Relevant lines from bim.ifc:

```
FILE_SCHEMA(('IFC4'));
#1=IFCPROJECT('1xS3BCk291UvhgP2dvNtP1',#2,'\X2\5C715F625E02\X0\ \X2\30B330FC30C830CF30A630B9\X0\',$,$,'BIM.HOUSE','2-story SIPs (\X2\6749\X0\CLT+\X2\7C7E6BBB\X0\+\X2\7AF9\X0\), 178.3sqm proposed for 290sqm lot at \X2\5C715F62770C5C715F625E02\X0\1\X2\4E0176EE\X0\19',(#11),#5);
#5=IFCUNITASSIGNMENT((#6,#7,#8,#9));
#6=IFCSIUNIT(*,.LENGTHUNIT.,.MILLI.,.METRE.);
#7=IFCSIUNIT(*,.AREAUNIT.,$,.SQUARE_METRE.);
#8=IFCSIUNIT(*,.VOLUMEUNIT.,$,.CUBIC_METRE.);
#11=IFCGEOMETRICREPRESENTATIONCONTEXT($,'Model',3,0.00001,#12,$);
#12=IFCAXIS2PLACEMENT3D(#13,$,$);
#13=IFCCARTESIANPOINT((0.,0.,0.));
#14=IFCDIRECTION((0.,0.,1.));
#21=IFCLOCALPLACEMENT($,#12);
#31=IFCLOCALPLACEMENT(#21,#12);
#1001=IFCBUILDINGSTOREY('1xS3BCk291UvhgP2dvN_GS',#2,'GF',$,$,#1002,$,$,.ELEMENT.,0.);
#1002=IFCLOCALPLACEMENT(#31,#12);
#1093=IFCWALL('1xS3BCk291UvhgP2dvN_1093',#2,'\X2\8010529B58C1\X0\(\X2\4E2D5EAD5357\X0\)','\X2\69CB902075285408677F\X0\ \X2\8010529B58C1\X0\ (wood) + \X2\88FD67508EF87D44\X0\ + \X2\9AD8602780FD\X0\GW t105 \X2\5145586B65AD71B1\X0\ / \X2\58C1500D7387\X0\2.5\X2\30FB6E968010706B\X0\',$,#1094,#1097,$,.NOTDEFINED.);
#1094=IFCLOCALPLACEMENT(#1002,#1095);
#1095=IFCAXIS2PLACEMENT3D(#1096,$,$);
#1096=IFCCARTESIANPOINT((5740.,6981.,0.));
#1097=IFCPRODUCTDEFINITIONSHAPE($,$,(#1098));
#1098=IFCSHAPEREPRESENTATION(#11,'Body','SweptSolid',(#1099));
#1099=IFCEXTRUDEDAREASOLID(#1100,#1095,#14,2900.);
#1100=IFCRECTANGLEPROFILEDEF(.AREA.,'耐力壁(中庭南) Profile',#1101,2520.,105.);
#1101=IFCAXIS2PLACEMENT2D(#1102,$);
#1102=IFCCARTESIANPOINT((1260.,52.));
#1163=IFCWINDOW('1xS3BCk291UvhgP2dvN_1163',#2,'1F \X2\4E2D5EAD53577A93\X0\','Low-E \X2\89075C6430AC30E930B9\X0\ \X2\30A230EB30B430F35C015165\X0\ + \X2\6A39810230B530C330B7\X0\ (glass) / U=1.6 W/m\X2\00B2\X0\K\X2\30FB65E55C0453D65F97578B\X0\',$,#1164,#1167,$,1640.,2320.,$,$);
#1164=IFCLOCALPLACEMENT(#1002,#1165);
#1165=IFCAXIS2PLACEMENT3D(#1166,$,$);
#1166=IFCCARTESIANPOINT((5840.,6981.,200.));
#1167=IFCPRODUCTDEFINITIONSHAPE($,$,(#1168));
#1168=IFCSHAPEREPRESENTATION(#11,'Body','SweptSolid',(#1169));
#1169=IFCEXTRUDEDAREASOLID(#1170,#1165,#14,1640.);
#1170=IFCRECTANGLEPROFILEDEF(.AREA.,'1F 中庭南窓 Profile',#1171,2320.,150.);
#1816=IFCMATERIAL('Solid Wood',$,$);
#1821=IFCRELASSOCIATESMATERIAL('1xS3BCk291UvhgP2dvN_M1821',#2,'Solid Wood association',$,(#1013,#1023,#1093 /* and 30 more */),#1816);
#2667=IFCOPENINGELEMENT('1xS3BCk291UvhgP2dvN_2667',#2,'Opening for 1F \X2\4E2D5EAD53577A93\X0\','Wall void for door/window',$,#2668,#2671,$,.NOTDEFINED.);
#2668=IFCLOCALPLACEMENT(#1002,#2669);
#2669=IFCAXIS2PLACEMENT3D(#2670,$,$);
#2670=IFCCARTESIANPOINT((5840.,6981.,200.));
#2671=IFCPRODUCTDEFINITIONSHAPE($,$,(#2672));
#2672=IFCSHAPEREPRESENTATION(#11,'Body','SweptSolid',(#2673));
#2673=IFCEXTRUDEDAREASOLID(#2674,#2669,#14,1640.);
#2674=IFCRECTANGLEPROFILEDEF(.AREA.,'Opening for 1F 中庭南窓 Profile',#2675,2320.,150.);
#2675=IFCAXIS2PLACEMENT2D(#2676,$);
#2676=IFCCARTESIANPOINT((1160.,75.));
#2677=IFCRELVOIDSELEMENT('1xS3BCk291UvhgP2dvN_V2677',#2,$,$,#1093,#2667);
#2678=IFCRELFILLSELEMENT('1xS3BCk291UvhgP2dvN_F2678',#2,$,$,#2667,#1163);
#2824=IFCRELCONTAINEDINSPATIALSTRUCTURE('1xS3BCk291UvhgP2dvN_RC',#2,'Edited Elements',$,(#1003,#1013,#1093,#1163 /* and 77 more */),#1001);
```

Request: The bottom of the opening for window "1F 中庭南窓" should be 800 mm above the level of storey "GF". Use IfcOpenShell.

```python
import numpy as np
import ifcopenshell
import ifcopenshell.api.geometry
import ifcopenshell.geom
import ifcopenshell.util.element
import ifcopenshell.util.placement
import ifcopenshell.util.shape
import ifcopenshell.util.unit

model = ifcopenshell.open("bim.ifc")
unit_scale = ifcopenshell.util.unit.calculate_unit_scale(model)

window = model.by_guid("1xS3BCk291UvhgP2dvN_1163")
opening = window.FillsVoids[0].RelatingOpeningElement
storey = ifcopenshell.util.element.get_container(window, ifc_class="IfcBuildingStorey")
level = ifcopenshell.util.placement.get_local_placement(storey.ObjectPlacement)[2, 3]

# The opening's origin need not be at the sill, so measure its lowest point.
shape = ifcopenshell.geom.create_shape(ifcopenshell.geom.settings(), opening)
bottom = ifcopenshell.util.shape.get_shape_bottom_elevation(shape, shape.geometry) / unit_scale
dz = level + 0.8 / unit_scale - bottom

shift = np.array([0.0, 0.0, dz])
# The window is not placed relative to its opening, so move both.
for product in (opening, window):
    matrix = ifcopenshell.util.placement.get_local_placement(product.ObjectPlacement)
    matrix[:3, 3] += shift
    ifcopenshell.api.geometry.edit_object_placement(model, product=product, matrix=matrix, is_si=False)

print(f"moved by {dz * unit_scale:+.3f} m")

model.write("bim-out.ifc")
```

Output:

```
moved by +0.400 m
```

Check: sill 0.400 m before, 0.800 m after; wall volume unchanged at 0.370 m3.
